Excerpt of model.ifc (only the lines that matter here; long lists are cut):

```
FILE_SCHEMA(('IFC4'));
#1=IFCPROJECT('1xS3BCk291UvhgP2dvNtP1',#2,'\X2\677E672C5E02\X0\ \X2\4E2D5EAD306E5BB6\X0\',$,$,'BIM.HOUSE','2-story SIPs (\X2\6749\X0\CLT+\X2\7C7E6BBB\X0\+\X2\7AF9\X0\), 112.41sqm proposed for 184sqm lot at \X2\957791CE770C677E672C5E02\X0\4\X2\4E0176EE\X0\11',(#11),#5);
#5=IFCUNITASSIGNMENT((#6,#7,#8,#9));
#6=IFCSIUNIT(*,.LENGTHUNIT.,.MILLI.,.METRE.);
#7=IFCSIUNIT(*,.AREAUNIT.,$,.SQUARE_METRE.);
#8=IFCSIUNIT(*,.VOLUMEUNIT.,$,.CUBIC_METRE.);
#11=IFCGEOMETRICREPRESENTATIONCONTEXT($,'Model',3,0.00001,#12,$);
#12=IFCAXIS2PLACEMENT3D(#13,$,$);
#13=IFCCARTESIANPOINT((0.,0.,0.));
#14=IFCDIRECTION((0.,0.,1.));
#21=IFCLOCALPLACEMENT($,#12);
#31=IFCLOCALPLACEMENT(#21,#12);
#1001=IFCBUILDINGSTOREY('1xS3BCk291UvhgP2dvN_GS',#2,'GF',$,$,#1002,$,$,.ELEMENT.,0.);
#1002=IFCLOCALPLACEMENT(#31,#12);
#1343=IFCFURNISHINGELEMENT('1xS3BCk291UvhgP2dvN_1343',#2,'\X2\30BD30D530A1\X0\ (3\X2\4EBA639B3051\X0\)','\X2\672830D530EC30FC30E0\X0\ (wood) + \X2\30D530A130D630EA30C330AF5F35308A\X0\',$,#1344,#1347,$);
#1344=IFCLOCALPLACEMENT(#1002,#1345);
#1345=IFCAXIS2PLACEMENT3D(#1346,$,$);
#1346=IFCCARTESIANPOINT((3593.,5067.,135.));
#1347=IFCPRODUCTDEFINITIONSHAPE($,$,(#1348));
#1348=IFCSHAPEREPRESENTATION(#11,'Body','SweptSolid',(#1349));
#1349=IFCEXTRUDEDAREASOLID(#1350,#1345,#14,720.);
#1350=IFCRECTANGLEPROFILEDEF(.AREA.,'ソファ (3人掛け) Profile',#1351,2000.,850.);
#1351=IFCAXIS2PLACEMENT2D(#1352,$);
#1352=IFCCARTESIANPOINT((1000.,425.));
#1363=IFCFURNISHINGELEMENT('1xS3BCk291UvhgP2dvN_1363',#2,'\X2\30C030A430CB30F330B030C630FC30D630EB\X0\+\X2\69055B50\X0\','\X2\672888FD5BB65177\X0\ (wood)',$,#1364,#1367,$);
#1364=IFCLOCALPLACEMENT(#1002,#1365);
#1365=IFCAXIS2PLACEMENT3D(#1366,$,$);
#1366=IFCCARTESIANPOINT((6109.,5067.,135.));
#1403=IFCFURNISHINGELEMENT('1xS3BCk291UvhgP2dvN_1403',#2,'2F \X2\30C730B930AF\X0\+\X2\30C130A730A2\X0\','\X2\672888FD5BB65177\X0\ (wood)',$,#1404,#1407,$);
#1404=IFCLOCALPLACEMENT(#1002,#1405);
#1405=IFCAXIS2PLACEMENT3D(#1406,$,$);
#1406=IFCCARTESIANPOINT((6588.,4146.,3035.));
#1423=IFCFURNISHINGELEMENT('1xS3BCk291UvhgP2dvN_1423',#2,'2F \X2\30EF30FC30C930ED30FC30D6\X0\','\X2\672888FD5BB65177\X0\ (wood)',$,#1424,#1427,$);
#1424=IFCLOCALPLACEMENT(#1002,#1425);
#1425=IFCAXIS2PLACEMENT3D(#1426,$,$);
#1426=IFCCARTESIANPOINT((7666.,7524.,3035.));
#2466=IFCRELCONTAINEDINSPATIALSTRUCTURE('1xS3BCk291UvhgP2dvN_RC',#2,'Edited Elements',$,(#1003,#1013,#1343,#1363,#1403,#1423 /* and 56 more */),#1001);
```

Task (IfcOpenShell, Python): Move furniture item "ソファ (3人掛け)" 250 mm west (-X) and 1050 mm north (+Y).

```python
import ifcopenshell
import ifcopenshell.api.geometry
import ifcopenshell.util.placement
import ifcopenshell.util.unit

model = ifcopenshell.open("model.ifc")
unit_scale = ifcopenshell.util.unit.calculate_unit_scale(model)

item = model.by_guid("1xS3BCk291UvhgP2dvN_1343")
matrix = ifcopenshell.util.placement.get_local_placement(item.ObjectPlacement)
matrix[0, 3] -= 0.25 / unit_scale
matrix[1, 3] += 1.05 / unit_scale
ifcopenshell.api.geometry.edit_object_placement(model, product=item, matrix=matrix, is_si=False)

print(ifcopenshell.util.placement.get_local_placement(item.ObjectPlacement).round(3) + 0.0)

model.write("model_edited.ifc")
```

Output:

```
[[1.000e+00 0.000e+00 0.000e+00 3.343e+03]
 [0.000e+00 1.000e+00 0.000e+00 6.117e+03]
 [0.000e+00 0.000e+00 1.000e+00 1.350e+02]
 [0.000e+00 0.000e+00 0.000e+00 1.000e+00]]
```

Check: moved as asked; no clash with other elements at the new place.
